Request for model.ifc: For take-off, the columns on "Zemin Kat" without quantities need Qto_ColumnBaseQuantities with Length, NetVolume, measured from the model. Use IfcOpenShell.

First a look at what the model holds.

```python
import ifcopenshell
import ifcopenshell.util.element
import ifcopenshell.util.unit

model = ifcopenshell.open("model.ifc")
print(model.schema)
for unit_type in ("LENGTHUNIT", "AREAUNIT", "VOLUMEUNIT"):
    print(unit_type, ifcopenshell.util.unit.calculate_unit_scale(model, unit_type))
storey = next(s for s in model.by_type("IfcBuildingStorey") if s.Name == "Zemin Kat")
columns = [e for e in ifcopenshell.util.element.get_decomposition(storey) if e.is_a("IfcColumn")]
for e in sorted(columns, key=lambda e: e.id()):
    print(e.id(), e.is_a(), e.Name, list(ifcopenshell.util.element.get_psets(e, qtos_only=True)), sep=" | ")
```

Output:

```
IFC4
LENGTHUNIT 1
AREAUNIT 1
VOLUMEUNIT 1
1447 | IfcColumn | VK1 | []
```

```python
import ifcopenshell
import ifcopenshell.api.pset
import ifcopenshell.geom
import ifcopenshell.util.element
import ifcopenshell.util.shape
import ifcopenshell.util.unit

model = ifcopenshell.open("model.ifc")
unit_scale = ifcopenshell.util.unit.calculate_unit_scale(model)
volume_scale = ifcopenshell.util.unit.calculate_unit_scale(model, "VOLUMEUNIT")
settings = ifcopenshell.geom.settings()

storey = next(s for s in model.by_type("IfcBuildingStorey") if s.Name == "Zemin Kat")
columns = [e for e in ifcopenshell.util.element.get_decomposition(storey) if e.is_a("IfcColumn")]

for e in sorted(columns, key=lambda e: e.id()):
    if ifcopenshell.util.element.get_psets(e, qtos_only=True, should_inherit=False):
        continue
    # Geometry comes back in metres, in the element's own axes.
    shape = ifcopenshell.geom.create_shape(settings, e)
    values = {
        "Length": ifcopenshell.util.shape.get_z(shape.geometry) / unit_scale,
        "NetVolume": ifcopenshell.util.shape.get_volume(shape.geometry) / volume_scale,
    }
    qto = ifcopenshell.api.pset.add_qto(model, product=e, name="Qto_ColumnBaseQuantities")
    ifcopenshell.api.pset.edit_qto(model, qto=qto, properties=values)
    print(e.id(), {k: round(v, 3) for k, v in values.items()})

model.write("model_updated.ifc")
```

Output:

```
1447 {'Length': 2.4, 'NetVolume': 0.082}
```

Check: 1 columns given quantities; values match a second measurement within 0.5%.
